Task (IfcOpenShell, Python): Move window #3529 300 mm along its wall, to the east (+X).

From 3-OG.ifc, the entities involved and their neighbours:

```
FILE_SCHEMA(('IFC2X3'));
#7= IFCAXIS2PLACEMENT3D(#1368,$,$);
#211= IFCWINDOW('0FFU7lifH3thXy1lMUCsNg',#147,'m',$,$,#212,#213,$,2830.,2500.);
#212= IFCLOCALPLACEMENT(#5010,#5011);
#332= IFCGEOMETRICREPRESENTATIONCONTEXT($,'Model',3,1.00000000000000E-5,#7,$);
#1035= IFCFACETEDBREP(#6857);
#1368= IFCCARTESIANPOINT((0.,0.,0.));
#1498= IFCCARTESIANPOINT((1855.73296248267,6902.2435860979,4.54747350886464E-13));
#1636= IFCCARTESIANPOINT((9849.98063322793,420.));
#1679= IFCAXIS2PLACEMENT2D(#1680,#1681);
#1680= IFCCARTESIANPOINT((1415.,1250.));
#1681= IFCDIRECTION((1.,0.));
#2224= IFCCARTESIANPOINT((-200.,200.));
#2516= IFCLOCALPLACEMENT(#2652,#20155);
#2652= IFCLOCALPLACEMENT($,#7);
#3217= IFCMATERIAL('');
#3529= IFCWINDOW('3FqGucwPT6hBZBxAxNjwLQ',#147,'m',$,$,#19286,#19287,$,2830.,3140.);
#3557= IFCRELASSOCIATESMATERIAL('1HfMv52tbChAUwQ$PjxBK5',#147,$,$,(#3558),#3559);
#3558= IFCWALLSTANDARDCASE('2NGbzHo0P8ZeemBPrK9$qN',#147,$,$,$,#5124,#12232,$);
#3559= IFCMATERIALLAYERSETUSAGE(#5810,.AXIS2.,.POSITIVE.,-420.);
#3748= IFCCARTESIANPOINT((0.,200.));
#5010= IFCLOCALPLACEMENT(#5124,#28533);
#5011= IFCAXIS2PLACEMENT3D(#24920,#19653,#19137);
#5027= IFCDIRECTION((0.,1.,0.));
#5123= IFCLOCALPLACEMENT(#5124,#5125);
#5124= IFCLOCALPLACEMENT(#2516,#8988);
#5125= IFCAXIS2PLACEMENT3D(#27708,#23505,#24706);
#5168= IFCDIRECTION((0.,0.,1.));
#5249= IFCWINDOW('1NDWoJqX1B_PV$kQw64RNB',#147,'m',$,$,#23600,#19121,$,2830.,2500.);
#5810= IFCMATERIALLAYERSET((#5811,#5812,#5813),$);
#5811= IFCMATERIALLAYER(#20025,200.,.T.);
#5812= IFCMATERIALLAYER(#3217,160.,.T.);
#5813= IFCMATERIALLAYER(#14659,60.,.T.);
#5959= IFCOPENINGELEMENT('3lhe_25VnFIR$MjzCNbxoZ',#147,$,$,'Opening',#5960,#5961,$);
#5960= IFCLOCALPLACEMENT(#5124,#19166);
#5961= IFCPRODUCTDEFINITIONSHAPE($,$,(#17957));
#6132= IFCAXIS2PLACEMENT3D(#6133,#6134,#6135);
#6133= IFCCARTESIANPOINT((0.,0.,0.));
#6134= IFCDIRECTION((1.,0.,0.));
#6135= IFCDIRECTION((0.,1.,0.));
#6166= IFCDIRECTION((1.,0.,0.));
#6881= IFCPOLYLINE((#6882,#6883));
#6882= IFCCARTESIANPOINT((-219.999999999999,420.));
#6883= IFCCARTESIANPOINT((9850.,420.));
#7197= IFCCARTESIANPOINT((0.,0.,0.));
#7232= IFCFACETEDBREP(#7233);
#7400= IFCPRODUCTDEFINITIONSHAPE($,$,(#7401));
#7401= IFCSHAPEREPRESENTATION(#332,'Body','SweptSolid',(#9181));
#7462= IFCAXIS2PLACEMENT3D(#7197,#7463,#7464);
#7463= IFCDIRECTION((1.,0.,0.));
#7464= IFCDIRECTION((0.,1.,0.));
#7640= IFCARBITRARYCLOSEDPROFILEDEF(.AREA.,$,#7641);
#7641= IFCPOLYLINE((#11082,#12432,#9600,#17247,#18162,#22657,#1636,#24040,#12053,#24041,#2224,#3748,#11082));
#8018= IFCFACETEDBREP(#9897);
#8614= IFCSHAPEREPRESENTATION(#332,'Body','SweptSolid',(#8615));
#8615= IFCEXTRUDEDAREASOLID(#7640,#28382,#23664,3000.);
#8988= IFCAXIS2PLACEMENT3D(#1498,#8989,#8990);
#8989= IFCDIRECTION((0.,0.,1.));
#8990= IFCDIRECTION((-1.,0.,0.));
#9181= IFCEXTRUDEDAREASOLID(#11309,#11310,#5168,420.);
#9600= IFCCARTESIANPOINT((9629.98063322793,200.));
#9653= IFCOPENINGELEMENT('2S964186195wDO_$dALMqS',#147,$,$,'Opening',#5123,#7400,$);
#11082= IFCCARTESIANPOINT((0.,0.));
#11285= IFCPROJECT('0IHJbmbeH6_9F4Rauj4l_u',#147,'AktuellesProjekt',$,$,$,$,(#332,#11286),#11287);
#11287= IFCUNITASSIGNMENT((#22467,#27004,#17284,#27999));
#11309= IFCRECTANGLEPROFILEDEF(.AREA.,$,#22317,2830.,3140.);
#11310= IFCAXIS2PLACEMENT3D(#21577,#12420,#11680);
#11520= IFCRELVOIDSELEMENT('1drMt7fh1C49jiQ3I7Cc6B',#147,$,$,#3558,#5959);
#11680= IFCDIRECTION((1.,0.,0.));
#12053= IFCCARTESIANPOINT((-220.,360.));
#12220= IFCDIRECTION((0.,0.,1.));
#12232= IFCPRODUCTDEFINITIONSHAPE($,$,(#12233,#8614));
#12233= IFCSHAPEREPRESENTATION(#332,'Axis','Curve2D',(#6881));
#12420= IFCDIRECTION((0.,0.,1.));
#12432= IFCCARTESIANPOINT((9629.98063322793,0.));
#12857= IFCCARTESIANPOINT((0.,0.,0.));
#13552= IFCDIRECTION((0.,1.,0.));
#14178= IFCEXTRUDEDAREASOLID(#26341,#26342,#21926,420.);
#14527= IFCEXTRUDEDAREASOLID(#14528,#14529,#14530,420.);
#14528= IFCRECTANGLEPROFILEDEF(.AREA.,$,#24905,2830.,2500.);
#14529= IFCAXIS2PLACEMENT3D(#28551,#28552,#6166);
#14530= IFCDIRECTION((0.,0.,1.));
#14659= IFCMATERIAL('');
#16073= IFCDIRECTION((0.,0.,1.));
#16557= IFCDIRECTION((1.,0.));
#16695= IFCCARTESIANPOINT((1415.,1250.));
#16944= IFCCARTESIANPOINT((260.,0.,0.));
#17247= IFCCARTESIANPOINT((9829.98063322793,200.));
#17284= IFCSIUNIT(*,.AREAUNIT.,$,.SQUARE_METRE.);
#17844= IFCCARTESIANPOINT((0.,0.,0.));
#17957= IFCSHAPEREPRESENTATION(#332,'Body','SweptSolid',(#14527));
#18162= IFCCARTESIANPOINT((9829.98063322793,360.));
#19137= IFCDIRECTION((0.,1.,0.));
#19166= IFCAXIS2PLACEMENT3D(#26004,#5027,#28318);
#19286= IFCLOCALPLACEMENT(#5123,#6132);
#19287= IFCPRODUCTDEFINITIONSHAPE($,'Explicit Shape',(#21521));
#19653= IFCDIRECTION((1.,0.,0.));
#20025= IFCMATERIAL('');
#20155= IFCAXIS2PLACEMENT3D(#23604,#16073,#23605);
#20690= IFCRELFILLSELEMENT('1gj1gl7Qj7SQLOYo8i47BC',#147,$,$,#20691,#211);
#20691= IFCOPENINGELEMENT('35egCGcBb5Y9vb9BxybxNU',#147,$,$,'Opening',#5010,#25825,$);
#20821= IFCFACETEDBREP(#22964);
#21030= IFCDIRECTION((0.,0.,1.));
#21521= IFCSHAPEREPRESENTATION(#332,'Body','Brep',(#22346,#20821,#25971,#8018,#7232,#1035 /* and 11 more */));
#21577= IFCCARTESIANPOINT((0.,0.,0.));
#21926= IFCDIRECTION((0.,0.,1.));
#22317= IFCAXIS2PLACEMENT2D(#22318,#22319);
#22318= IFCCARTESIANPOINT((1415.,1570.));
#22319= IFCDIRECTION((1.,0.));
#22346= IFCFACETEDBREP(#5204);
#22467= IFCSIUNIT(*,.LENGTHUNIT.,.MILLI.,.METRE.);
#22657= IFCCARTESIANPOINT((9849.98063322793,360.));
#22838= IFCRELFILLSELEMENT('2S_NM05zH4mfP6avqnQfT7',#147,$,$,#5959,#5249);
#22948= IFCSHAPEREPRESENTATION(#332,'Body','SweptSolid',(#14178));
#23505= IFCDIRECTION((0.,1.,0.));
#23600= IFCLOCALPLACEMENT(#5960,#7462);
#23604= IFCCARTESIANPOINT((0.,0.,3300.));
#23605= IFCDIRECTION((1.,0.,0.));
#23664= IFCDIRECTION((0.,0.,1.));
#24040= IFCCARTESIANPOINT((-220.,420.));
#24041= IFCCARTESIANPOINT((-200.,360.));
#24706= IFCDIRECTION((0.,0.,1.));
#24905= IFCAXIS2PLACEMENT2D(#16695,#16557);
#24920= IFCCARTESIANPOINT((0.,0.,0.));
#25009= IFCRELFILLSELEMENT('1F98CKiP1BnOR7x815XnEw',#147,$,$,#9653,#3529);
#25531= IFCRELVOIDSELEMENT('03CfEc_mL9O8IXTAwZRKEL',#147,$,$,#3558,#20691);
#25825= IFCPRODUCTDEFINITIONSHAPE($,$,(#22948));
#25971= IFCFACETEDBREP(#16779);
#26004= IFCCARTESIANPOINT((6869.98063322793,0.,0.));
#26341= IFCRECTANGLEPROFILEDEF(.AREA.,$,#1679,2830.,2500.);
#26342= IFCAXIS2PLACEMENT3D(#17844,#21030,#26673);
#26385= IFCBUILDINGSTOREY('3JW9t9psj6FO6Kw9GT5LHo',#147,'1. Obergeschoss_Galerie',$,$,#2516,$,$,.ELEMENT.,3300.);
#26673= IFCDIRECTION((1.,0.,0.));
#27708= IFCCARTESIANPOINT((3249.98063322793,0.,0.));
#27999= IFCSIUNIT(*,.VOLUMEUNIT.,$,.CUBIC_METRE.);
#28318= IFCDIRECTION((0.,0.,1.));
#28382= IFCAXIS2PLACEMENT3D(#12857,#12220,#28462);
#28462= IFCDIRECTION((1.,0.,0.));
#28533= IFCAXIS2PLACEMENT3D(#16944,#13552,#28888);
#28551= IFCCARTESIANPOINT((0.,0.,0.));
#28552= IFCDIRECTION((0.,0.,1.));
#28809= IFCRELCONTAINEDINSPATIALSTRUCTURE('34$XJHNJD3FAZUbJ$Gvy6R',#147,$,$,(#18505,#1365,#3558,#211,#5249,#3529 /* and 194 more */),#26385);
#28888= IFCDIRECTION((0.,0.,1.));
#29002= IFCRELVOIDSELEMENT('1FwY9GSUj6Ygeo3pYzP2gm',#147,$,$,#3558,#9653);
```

```python
import ifcopenshell
import ifcopenshell.api.geometry
import ifcopenshell.util.placement
import ifcopenshell.util.unit

model = ifcopenshell.open("3-OG.ifc")
unit_scale = ifcopenshell.util.unit.calculate_unit_scale(model)

window = model.by_guid("3FqGucwPT6hBZBxAxNjwLQ")
opening = window.FillsVoids[0].RelatingOpeningElement
wall = opening.VoidsElements[0].RelatingBuildingElement

wall_matrix = ifcopenshell.util.placement.get_local_placement(wall.ObjectPlacement)
shift = wall_matrix[:3, 0] * -0.3 / unit_scale
before = ifcopenshell.util.placement.get_local_placement(window.ObjectPlacement)[:3, 3].copy()

# The window is placed relative to its opening, so it follows when the opening moves.
matrix = ifcopenshell.util.placement.get_local_placement(opening.ObjectPlacement)
matrix[:3, 3] += shift
ifcopenshell.api.geometry.edit_object_placement(
    model, product=opening, matrix=matrix, is_si=False, should_transform_children=True
)

after = ifcopenshell.util.placement.get_local_placement(window.ObjectPlacement)[:3, 3]
print("window moved by", (after - before).round(3) + 0.0)

model.write("3-OG_edited.ifc")
```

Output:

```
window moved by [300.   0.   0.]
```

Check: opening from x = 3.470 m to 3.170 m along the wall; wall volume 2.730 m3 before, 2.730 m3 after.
